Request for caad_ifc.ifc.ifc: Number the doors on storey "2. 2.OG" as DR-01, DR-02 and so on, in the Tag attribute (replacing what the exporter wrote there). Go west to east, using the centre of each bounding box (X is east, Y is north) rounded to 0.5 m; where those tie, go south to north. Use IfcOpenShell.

First a look at what the model holds.

```python
import ifcopenshell
import ifcopenshell.util.element
import ifcopenshell.util.placement

model = ifcopenshell.open("caad_ifc.ifc.ifc")
print(model.schema)
storey = next(s for s in model.by_type("IfcBuildingStorey") if s.Name == "2. 2.OG")
doors = [e for e in ifcopenshell.util.element.get_decomposition(storey) if e.is_a("IfcDoor")]
for e in sorted(doors, key=lambda e: e.id()):
    origin = ifcopenshell.util.placement.get_local_placement(e.ObjectPlacement)[:3, 3]
    print(e.id(), e.Tag, e.Name, origin.round(2) + 0.0, sep=" | ")
```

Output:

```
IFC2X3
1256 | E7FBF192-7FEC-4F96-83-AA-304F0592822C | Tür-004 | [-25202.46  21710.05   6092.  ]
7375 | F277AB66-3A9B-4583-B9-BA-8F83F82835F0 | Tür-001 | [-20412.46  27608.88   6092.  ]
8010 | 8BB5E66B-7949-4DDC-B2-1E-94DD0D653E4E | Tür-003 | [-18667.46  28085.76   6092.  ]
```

```python
import ifcopenshell
import ifcopenshell.geom
import ifcopenshell.util.element
import ifcopenshell.util.shape

model = ifcopenshell.open("caad_ifc.ifc.ifc")
settings = ifcopenshell.geom.settings()
settings.set("use-world-coords", True)


def centre(element):
    shape = ifcopenshell.geom.create_shape(settings, element)
    return ifcopenshell.util.shape.get_bbox_centroid(shape.geometry)


storey = next(s for s in model.by_type("IfcBuildingStorey") if s.Name == "2. 2.OG")
doors = [e for e in ifcopenshell.util.element.get_decomposition(storey) if e.is_a("IfcDoor")]

# Insertion points can sit at a corner or the storey origin, so sort by the geometry (in metres).
centres = {e: centre(e) for e in doors}
doors.sort(key=lambda e: (round(centres[e][0] / 0.5), centres[e][1]))

for i, e in enumerate(doors, start=1):
    number = f"DR-{i:02d}"
    e.Tag = number
    print(e.id(), number)

model.write("caad_ifc.ifc_rev.ifc")
```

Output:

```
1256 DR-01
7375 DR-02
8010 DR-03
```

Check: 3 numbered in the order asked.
